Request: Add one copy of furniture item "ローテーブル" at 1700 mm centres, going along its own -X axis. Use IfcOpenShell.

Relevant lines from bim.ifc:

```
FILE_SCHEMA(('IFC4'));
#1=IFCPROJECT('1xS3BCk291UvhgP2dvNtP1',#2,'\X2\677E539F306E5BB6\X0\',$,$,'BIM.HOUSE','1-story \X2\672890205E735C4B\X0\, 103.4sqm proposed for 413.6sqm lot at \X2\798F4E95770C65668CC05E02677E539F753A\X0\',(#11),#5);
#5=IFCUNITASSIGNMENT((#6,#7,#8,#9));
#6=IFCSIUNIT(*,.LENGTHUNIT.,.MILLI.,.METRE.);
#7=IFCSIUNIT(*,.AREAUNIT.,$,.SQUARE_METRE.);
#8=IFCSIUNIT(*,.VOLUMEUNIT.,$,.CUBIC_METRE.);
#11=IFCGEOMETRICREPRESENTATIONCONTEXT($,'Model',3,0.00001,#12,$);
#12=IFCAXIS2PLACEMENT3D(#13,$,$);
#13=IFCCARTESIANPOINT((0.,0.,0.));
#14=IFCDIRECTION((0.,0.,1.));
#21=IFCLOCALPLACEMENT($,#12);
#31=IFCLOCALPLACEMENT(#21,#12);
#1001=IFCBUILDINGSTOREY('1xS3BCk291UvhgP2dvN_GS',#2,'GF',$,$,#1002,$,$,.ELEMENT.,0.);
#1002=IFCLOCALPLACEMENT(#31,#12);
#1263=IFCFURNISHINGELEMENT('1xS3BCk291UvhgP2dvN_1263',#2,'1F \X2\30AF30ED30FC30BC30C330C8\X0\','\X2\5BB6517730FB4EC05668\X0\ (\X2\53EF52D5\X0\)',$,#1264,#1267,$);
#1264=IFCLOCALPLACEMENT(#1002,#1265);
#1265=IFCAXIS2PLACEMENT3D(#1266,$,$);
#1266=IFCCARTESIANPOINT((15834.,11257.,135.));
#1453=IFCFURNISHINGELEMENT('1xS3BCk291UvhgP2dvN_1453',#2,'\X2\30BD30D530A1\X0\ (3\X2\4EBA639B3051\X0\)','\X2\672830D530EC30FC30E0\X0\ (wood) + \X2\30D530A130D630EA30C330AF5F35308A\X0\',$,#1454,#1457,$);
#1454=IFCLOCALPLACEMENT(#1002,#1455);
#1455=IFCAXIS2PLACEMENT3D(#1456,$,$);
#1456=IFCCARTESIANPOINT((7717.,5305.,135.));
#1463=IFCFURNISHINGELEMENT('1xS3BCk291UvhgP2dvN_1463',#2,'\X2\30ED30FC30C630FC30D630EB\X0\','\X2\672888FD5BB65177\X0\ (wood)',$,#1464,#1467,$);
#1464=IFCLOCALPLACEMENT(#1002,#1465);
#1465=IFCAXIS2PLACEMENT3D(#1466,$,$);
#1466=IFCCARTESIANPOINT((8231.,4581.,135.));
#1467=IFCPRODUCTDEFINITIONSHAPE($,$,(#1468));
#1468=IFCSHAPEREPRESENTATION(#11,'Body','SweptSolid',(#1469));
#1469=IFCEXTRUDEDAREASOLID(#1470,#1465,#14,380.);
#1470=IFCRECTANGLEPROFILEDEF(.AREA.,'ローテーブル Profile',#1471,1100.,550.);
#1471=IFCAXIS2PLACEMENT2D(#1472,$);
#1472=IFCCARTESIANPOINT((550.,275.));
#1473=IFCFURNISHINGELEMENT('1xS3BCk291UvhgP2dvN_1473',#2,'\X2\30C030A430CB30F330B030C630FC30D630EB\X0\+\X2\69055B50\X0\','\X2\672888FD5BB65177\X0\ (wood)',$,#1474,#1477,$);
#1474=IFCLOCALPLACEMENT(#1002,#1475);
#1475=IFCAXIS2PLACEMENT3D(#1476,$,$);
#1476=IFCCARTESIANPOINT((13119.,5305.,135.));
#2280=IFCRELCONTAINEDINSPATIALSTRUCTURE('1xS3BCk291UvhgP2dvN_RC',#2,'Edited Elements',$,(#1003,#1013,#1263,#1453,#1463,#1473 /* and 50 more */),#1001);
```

```python
import ifcopenshell
import ifcopenshell.api.geometry
import ifcopenshell.api.root
import ifcopenshell.util.element
import ifcopenshell.util.placement

model = ifcopenshell.open("bim.ifc")


def reuse_history(source, copy):
    """copy_class also copies each property set's owner history, people and application; keep the originals."""
    for rel in copy.IsDefinedBy:
        if rel.is_a("IfcRelDefinesByProperties") and (history := rel.RelatingPropertyDefinition.OwnerHistory):
            rel.RelatingPropertyDefinition.OwnerHistory = source.OwnerHistory
            ifcopenshell.util.element.remove_deep2(model, history)


source = model.by_guid("1xS3BCk291UvhgP2dvN_1463")
base = ifcopenshell.util.placement.get_local_placement(source.ObjectPlacement)
step = -base[:3, 0] * 1700.0

for i in range(1, 2):
    copy = ifcopenshell.api.root.copy_class(model, product=source)
    copy.Representation = ifcopenshell.util.element.copy_deep(
        model, source.Representation, exclude=["IfcGeometricRepresentationContext", "IfcRepresentationMap"]
    )
    reuse_history(source, copy)
    matrix = base.copy()
    matrix[:3, 3] += i * step
    print("added at", matrix[:3, 3].round(3) + 0.0)
    ifcopenshell.api.geometry.edit_object_placement(model, product=copy, matrix=matrix, is_si=False)

model.write("bim-out.ifc")
```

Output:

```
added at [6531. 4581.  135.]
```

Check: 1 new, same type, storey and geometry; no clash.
